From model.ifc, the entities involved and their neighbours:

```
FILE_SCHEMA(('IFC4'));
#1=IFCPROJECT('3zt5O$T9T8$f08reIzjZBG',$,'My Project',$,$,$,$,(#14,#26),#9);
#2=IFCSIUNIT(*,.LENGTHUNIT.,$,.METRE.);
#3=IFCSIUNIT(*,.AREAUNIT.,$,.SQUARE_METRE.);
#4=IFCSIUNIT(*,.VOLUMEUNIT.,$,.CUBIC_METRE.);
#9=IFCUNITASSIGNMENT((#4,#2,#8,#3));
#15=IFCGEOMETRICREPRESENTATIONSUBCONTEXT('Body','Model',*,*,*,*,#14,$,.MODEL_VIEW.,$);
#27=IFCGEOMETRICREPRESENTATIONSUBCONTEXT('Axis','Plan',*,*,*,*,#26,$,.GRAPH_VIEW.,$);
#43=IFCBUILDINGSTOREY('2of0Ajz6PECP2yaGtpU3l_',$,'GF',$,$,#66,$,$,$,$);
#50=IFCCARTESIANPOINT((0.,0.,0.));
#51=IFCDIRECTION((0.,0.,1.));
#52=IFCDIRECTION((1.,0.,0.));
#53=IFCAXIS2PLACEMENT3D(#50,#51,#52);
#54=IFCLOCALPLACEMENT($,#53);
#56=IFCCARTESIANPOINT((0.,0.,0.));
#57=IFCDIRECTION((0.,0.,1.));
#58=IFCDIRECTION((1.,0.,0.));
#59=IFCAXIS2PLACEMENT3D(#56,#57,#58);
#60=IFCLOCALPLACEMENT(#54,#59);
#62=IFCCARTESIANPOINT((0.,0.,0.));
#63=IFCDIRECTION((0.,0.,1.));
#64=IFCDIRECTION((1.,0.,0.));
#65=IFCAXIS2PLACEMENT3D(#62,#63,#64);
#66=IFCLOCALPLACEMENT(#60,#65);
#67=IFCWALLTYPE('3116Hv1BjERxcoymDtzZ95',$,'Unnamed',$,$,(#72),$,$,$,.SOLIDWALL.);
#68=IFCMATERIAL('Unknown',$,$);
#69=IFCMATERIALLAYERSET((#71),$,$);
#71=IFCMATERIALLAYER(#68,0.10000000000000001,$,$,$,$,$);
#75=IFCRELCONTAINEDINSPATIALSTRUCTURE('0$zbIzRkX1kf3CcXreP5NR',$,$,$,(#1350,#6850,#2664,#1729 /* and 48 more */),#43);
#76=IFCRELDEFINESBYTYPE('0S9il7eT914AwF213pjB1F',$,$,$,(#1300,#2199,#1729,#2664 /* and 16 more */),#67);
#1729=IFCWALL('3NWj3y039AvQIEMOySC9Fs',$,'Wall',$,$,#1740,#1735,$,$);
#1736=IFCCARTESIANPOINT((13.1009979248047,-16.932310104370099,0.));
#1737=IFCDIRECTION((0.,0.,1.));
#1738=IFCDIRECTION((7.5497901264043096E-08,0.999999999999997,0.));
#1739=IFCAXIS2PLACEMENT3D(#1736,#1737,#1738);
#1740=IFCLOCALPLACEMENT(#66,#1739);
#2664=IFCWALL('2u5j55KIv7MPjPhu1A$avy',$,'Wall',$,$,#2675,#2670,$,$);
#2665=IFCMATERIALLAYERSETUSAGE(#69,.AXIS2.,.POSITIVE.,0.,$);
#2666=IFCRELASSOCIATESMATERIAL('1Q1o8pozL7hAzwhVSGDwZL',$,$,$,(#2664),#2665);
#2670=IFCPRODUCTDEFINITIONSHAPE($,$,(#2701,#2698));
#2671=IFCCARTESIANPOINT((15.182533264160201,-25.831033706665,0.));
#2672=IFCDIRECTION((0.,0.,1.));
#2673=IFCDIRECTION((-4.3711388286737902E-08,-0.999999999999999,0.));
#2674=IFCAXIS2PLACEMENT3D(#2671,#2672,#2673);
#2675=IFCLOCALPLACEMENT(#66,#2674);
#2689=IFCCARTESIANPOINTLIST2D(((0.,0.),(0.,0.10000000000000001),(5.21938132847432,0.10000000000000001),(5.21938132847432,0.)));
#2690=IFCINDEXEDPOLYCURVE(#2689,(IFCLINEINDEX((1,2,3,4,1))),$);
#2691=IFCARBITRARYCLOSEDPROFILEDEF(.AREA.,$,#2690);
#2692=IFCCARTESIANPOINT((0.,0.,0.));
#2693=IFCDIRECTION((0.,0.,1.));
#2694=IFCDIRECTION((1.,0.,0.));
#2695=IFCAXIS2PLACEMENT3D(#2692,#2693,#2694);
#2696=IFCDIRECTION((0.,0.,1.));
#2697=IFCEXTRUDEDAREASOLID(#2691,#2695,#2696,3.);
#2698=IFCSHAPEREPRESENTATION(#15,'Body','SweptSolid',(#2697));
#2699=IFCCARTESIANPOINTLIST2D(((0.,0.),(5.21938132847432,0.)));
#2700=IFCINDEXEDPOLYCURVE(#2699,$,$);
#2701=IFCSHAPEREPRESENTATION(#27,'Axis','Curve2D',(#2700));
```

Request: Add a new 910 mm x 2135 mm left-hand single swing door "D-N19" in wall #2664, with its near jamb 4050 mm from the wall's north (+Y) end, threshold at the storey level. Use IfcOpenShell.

```python
import numpy as np
import ifcopenshell
import ifcopenshell.api.feature
import ifcopenshell.api.geometry
import ifcopenshell.api.root
import ifcopenshell.api.spatial
import ifcopenshell.geom
import ifcopenshell.util.element
import ifcopenshell.util.placement
import ifcopenshell.util.representation
import ifcopenshell.util.shape
import ifcopenshell.util.unit

model = ifcopenshell.open("model.ifc")
unit_scale = ifcopenshell.util.unit.calculate_unit_scale(model)
settings = ifcopenshell.geom.settings()


def volume(element):
    """Net volume in cubic metres, openings subtracted."""
    shape = ifcopenshell.geom.create_shape(settings, element)
    return ifcopenshell.util.shape.get_volume(shape.geometry)


wall = model.by_id(2664)
storey = ifcopenshell.util.element.get_container(wall, ifc_class="IfcBuildingStorey")
context = ifcopenshell.util.representation.get_context(model, "Model", "Body", "MODEL_VIEW")
before = volume(wall)

width, height, from_end, sill = 0.91, 2.135, 4.05, 0.0  # metres

# The wall runs along its own X axis, and the end named is its -X end.
wall_shape = ifcopenshell.geom.create_shape(settings, wall)
x, y, z = ifcopenshell.util.shape.get_vertices(wall_shape.geometry).T
start = x.min() + from_end
face, thickness = float(y.min()), float(y.max() - y.min())
wall_matrix = ifcopenshell.util.placement.get_local_placement(wall.ObjectPlacement)
level = ifcopenshell.util.placement.get_local_placement(storey.ObjectPlacement)[2, 3]


def in_wall(x, y):
    """Placement at x, y metres in the wall's axes, at sill height."""
    matrix = wall_matrix.copy()
    matrix[:, 3] = wall_matrix @ np.array([x / unit_scale, y / unit_scale, 0.0, 1.0])
    matrix[2, 3] = level + sill / unit_scale
    return matrix


# Opening: a box that overshoots both wall faces by 50 mm.
opening = ifcopenshell.api.root.create_entity(model, ifc_class="IfcOpeningElement", predefined_type="OPENING")
box = ifcopenshell.api.geometry.add_wall_representation(
    model, context=context, length=width, height=height, thickness=thickness + 0.1
)
ifcopenshell.api.geometry.assign_representation(model, product=opening, representation=box)
ifcopenshell.api.geometry.edit_object_placement(model, product=opening, matrix=in_wall(start, face - 0.05), is_si=False)
ifcopenshell.api.feature.add_feature(model, feature=opening, element=wall)

door = ifcopenshell.api.root.create_entity(model, ifc_class="IfcDoor", name="D-N19", predefined_type="DOOR")
door.OverallWidth, door.OverallHeight = width / unit_scale, height / unit_scale
door.OperationType = "SINGLE_SWING_LEFT"
body = ifcopenshell.api.geometry.add_door_representation(
    model,
    context=context,
    overall_width=door.OverallWidth,
    overall_height=door.OverallHeight,
    operation_type="SINGLE_SWING_LEFT",
    lining_properties={"LiningDepth": thickness / unit_scale, "ThresholdDepth": thickness / unit_scale},
)
ifcopenshell.api.geometry.assign_representation(model, product=door, representation=body)
ifcopenshell.api.spatial.assign_container(model, products=[door], relating_structure=storey)
ifcopenshell.api.feature.add_filling(model, opening=opening, element=door)

# The lining spans the wall, so the door starts at the wall face.
ifcopenshell.api.geometry.edit_object_placement(model, product=door, matrix=in_wall(start, face), is_si=False)

after = volume(wall)

print(f"wall volume {before:.3f} -> {after:.3f} m3")

model.write("model_edited.ifc")
```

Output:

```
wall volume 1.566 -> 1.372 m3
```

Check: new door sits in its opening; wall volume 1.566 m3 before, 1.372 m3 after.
